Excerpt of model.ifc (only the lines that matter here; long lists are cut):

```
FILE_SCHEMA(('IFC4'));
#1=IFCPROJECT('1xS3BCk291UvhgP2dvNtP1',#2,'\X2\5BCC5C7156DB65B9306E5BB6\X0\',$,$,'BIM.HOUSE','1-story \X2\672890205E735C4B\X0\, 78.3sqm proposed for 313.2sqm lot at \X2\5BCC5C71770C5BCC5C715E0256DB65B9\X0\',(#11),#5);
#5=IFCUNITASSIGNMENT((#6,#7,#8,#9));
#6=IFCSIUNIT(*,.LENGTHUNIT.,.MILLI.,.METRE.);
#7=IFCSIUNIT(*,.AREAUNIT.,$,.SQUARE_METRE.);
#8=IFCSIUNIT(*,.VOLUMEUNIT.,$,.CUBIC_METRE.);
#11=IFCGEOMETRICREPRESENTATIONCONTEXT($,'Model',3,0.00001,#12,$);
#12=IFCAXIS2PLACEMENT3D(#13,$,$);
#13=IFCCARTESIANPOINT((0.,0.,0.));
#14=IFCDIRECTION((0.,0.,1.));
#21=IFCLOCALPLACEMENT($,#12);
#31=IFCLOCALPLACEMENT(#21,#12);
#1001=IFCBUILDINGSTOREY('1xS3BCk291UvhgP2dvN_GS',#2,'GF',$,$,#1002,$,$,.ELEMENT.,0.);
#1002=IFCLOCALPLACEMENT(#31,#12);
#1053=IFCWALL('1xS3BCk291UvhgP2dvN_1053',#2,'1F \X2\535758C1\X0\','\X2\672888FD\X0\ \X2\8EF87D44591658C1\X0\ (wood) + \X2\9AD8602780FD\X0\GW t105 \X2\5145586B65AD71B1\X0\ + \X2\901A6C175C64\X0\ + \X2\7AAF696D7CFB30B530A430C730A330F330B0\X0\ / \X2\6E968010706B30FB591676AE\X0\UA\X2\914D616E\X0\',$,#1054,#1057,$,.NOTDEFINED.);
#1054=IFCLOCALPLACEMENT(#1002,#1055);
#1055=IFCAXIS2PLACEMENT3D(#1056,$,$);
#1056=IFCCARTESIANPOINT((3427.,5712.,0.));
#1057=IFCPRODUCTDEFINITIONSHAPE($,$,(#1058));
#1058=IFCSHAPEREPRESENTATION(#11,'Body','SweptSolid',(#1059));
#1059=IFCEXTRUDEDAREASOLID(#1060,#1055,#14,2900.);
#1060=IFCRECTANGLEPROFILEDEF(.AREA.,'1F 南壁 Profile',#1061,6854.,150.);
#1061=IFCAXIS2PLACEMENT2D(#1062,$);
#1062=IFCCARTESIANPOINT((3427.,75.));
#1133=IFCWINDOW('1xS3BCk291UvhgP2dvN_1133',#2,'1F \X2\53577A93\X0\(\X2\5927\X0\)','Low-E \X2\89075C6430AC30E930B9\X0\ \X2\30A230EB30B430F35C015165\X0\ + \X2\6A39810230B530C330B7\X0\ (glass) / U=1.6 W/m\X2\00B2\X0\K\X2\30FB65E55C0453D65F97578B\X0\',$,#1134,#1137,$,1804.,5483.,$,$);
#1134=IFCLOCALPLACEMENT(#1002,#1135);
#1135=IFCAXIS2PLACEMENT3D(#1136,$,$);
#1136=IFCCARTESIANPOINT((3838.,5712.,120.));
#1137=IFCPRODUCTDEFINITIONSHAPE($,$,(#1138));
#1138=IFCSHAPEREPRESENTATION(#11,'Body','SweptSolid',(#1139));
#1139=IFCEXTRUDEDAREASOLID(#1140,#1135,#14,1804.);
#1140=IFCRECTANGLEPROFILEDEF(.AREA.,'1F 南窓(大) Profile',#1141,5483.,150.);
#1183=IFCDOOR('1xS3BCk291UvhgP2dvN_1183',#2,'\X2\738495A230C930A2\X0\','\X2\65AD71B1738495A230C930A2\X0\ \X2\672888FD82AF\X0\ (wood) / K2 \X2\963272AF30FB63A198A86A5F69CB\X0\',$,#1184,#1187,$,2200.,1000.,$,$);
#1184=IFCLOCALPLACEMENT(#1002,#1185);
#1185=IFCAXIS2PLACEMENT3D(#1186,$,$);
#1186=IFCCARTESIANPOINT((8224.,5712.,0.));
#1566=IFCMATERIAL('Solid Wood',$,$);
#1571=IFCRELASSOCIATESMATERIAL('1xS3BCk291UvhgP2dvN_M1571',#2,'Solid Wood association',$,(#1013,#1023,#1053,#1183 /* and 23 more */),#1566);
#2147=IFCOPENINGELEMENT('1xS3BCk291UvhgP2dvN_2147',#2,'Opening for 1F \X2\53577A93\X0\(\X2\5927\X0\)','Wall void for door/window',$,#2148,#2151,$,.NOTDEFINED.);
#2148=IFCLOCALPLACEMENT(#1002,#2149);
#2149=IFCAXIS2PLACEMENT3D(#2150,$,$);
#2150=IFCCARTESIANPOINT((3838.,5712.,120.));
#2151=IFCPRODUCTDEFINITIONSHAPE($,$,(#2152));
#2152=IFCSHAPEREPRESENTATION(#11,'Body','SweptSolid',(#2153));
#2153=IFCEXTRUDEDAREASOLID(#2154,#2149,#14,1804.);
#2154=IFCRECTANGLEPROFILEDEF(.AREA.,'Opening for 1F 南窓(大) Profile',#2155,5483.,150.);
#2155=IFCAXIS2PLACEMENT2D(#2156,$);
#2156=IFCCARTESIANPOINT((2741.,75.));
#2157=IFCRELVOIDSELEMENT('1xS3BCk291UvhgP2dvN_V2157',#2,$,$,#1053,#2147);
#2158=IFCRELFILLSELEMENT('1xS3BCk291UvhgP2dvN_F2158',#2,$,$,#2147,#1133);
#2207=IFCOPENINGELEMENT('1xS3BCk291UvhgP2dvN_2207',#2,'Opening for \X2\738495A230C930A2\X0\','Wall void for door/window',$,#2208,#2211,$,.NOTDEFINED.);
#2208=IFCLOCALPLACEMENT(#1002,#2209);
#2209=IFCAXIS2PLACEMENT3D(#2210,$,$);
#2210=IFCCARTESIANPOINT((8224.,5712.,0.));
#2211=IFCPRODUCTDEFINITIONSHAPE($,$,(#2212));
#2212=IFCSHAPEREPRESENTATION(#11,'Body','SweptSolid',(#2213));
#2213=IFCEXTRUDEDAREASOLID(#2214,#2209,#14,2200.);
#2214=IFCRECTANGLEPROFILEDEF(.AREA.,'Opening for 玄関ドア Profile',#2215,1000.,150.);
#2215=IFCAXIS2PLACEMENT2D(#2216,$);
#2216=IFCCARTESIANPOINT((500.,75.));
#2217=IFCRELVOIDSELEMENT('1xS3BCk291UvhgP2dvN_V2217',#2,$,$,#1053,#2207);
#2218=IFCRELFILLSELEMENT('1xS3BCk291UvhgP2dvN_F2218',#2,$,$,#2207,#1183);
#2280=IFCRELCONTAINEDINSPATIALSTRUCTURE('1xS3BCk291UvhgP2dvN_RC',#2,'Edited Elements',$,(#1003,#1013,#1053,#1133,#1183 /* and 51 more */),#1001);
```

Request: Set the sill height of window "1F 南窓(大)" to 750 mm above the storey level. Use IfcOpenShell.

```python
import numpy as np
import ifcopenshell
import ifcopenshell.api.geometry
import ifcopenshell.geom
import ifcopenshell.util.element
import ifcopenshell.util.placement
import ifcopenshell.util.shape
import ifcopenshell.util.unit

model = ifcopenshell.open("model.ifc")
unit_scale = ifcopenshell.util.unit.calculate_unit_scale(model)

window = model.by_guid("1xS3BCk291UvhgP2dvN_1133")
opening = window.FillsVoids[0].RelatingOpeningElement
storey = ifcopenshell.util.element.get_container(window, ifc_class="IfcBuildingStorey")
level = ifcopenshell.util.placement.get_local_placement(storey.ObjectPlacement)[2, 3]

# The opening's origin need not be at the sill, so measure its lowest point.
shape = ifcopenshell.geom.create_shape(ifcopenshell.geom.settings(), opening)
bottom = ifcopenshell.util.shape.get_shape_bottom_elevation(shape, shape.geometry) / unit_scale
dz = level + 0.75 / unit_scale - bottom

shift = np.array([0.0, 0.0, dz])
# The window is not placed relative to its opening, so move both.
for product in (opening, window):
    matrix = ifcopenshell.util.placement.get_local_placement(product.ObjectPlacement)
    matrix[:3, 3] += shift
    ifcopenshell.api.geometry.edit_object_placement(model, product=product, matrix=matrix, is_si=False)

print(f"moved by {dz * unit_scale:+.3f} m")

model.write("model_v2.ifc")
```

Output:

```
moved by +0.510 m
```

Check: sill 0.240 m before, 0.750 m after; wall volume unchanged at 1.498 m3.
